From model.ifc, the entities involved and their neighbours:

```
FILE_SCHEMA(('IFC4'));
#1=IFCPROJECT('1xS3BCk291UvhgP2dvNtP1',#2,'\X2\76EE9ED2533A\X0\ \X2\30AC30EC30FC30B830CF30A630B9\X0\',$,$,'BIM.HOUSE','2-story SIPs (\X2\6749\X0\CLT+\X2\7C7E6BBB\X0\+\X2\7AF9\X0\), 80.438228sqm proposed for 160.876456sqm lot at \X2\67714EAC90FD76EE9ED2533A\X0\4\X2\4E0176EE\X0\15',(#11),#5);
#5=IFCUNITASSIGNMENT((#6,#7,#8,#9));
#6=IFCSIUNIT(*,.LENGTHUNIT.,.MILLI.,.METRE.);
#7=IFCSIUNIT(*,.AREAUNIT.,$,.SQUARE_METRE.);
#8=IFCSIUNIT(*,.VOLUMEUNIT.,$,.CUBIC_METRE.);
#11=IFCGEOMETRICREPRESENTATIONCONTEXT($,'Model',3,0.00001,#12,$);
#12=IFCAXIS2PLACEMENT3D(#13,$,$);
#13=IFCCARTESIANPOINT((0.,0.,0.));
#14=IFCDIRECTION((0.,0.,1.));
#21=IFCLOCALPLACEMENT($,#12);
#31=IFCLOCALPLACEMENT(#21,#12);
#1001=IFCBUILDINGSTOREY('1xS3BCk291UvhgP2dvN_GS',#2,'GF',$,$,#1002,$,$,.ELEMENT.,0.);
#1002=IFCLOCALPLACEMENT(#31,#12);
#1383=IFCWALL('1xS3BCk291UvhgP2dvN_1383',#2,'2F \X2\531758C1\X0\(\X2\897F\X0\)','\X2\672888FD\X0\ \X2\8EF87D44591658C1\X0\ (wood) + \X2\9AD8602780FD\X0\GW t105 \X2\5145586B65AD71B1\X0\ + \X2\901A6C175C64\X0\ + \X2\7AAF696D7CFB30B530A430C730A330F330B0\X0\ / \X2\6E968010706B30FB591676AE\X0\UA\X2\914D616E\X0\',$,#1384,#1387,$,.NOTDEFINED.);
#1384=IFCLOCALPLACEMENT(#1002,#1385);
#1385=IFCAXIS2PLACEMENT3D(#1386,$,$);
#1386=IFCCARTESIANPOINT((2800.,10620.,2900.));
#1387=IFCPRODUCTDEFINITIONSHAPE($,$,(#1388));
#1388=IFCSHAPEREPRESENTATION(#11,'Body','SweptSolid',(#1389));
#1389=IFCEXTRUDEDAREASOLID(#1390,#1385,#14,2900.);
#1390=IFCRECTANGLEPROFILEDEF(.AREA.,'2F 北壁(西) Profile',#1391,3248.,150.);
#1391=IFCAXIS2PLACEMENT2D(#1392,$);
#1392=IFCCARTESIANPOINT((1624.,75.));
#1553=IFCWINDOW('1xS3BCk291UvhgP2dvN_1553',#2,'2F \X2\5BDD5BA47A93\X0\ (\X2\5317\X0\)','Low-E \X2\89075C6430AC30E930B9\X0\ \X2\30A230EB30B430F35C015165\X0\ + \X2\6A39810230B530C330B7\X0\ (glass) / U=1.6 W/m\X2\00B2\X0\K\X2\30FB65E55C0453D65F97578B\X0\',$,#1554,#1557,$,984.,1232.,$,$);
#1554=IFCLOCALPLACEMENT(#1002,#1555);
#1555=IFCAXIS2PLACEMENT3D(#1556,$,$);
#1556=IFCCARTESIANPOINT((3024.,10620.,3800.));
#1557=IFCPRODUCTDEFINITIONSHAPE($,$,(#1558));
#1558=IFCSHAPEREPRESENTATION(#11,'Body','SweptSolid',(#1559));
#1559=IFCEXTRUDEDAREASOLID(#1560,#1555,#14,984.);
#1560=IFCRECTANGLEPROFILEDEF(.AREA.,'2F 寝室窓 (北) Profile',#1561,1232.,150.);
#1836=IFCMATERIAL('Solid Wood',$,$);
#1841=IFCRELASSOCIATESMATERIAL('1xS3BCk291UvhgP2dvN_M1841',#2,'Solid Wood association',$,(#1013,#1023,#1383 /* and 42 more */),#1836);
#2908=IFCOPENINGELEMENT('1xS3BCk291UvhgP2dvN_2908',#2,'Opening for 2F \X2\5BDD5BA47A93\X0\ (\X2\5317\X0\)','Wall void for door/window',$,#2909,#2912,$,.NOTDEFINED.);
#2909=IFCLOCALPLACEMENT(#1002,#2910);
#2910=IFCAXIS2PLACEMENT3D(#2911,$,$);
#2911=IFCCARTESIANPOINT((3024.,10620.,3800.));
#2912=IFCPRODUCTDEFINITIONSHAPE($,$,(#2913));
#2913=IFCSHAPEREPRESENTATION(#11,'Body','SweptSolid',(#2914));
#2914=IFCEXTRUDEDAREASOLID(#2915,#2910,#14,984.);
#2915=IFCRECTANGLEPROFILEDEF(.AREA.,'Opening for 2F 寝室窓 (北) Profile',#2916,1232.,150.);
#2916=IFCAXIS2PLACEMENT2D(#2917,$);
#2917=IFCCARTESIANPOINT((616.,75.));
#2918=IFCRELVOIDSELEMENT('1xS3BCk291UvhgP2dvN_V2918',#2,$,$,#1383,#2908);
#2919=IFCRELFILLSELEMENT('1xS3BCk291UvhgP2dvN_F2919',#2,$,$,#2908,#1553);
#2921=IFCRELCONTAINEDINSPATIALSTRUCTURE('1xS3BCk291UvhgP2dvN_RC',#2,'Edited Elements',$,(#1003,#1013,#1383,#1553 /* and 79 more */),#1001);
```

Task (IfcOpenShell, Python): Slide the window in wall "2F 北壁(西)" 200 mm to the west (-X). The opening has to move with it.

```python
import ifcopenshell
import ifcopenshell.api.geometry
import ifcopenshell.util.placement

model = ifcopenshell.open("model.ifc")

window = model.by_guid("1xS3BCk291UvhgP2dvN_1553")
opening = window.FillsVoids[0].RelatingOpeningElement
wall = opening.VoidsElements[0].RelatingBuildingElement

wall_matrix = ifcopenshell.util.placement.get_local_placement(wall.ObjectPlacement)
shift = wall_matrix[:3, 0] * -200.0
before = ifcopenshell.util.placement.get_local_placement(window.ObjectPlacement)[:3, 3].copy()

# The window is not placed relative to its opening, so move both.
for product in (opening, window):
    matrix = ifcopenshell.util.placement.get_local_placement(product.ObjectPlacement)
    matrix[:3, 3] += shift
    ifcopenshell.api.geometry.edit_object_placement(model, product=product, matrix=matrix, is_si=False)

after = ifcopenshell.util.placement.get_local_placement(window.ObjectPlacement)[:3, 3]
print("window moved by", (after - before).round(3) + 0.0)

model.write("model_v2.ifc")
```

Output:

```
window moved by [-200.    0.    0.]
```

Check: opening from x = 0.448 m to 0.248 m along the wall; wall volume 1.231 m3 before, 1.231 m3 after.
